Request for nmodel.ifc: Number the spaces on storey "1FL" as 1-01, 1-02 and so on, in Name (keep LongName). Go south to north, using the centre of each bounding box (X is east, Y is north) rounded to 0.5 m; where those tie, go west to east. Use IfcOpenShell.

First a look at what the model holds.

```python
import ifcopenshell
import ifcopenshell.util.element
import ifcopenshell.util.placement

model = ifcopenshell.open("nmodel.ifc")
print(model.schema)
storey = next(s for s in model.by_type("IfcBuildingStorey") if s.Name == "1FL")
spaces = [e for e in ifcopenshell.util.element.get_decomposition(storey) if e.is_a("IfcSpace")]
for e in sorted(spaces, key=lambda e: e.id()):
    origin = ifcopenshell.util.placement.get_local_placement(e.ObjectPlacement)[:3, 3]
    print(e.id(), e.Name, e.LongName, origin.round(2) + 0.0, sep=" | ")
```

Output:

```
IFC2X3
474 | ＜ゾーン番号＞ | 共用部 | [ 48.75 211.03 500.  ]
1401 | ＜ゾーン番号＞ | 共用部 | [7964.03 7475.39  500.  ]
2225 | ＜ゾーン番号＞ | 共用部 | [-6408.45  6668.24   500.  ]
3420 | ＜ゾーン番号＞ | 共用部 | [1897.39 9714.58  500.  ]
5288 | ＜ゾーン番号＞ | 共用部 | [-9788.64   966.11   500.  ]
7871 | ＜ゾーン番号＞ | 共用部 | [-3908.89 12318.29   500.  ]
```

```python
import ifcopenshell
import ifcopenshell.geom
import ifcopenshell.util.element
import ifcopenshell.util.shape

model = ifcopenshell.open("nmodel.ifc")
settings = ifcopenshell.geom.settings()
settings.set("use-world-coords", True)


def centre(element):
    shape = ifcopenshell.geom.create_shape(settings, element)
    return ifcopenshell.util.shape.get_bbox_centroid(shape.geometry)


storey = next(s for s in model.by_type("IfcBuildingStorey") if s.Name == "1FL")
spaces = [e for e in ifcopenshell.util.element.get_decomposition(storey) if e.is_a("IfcSpace")]

# Insertion points can sit at a corner or the storey origin, so sort by the geometry (in metres).
centres = {e: centre(e) for e in spaces}
spaces.sort(key=lambda e: (round(centres[e][1] / 0.5), centres[e][0]))

for i, e in enumerate(spaces, start=1):
    number = f"1-{i:02d}"
    e.Name = number
    print(e.id(), number)

model.write("nmodel_rev.ifc")
```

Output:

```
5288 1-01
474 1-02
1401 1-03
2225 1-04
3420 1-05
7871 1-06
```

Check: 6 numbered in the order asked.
